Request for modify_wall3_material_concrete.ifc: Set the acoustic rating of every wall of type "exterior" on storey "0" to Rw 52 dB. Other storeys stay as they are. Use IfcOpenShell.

First a look at what the model holds.

```python
import ifcopenshell
import ifcopenshell.util.element

model = ifcopenshell.open("modify_wall3_material_concrete.ifc")
print(model.schema)
storey = next(s for s in model.by_type("IfcBuildingStorey") if s.Name == "0")
walls = [e for e in ifcopenshell.util.element.get_decomposition(storey) if e.is_a("IfcWall")]
seen = {}
for e in walls:
    element_type = ifcopenshell.util.element.get_type(e)
    key = (element_type.Name if element_type != e and element_type else None, ifcopenshell.util.element.get_pset(e, "Pset_WallCommon", "AcousticRating"))
    seen[key] = seen.get(key, 0) + 1
for (name, value), count in sorted(seen.items(), key=str):
    print(count, "x", name, "|", value)
```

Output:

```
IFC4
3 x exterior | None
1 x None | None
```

```python
import ifcopenshell
import ifcopenshell.api.pset
import ifcopenshell.util.element

model = ifcopenshell.open("modify_wall3_material_concrete.ifc")

storey = next(s for s in model.by_type("IfcBuildingStorey") if s.Name == "0")
walls = [e for e in ifcopenshell.util.element.get_decomposition(storey) if e.is_a("IfcWall")]

count = 0
for e in walls:
    element_type = ifcopenshell.util.element.get_type(e)
    if element_type in (None, e) or element_type.Name != "exterior":
        continue
    # add_pset returns the element's existing set when there is one.
    pset = ifcopenshell.api.pset.add_pset(model, product=e, name="Pset_WallCommon")
    ifcopenshell.api.pset.edit_pset(model, pset=pset, properties={"AcousticRating": "Rw 52 dB"})
    count += 1

print(count, "walls updated")

model.write("modify_wall3_material_concrete_rev.ifc")
```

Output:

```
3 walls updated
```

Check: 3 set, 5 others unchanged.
